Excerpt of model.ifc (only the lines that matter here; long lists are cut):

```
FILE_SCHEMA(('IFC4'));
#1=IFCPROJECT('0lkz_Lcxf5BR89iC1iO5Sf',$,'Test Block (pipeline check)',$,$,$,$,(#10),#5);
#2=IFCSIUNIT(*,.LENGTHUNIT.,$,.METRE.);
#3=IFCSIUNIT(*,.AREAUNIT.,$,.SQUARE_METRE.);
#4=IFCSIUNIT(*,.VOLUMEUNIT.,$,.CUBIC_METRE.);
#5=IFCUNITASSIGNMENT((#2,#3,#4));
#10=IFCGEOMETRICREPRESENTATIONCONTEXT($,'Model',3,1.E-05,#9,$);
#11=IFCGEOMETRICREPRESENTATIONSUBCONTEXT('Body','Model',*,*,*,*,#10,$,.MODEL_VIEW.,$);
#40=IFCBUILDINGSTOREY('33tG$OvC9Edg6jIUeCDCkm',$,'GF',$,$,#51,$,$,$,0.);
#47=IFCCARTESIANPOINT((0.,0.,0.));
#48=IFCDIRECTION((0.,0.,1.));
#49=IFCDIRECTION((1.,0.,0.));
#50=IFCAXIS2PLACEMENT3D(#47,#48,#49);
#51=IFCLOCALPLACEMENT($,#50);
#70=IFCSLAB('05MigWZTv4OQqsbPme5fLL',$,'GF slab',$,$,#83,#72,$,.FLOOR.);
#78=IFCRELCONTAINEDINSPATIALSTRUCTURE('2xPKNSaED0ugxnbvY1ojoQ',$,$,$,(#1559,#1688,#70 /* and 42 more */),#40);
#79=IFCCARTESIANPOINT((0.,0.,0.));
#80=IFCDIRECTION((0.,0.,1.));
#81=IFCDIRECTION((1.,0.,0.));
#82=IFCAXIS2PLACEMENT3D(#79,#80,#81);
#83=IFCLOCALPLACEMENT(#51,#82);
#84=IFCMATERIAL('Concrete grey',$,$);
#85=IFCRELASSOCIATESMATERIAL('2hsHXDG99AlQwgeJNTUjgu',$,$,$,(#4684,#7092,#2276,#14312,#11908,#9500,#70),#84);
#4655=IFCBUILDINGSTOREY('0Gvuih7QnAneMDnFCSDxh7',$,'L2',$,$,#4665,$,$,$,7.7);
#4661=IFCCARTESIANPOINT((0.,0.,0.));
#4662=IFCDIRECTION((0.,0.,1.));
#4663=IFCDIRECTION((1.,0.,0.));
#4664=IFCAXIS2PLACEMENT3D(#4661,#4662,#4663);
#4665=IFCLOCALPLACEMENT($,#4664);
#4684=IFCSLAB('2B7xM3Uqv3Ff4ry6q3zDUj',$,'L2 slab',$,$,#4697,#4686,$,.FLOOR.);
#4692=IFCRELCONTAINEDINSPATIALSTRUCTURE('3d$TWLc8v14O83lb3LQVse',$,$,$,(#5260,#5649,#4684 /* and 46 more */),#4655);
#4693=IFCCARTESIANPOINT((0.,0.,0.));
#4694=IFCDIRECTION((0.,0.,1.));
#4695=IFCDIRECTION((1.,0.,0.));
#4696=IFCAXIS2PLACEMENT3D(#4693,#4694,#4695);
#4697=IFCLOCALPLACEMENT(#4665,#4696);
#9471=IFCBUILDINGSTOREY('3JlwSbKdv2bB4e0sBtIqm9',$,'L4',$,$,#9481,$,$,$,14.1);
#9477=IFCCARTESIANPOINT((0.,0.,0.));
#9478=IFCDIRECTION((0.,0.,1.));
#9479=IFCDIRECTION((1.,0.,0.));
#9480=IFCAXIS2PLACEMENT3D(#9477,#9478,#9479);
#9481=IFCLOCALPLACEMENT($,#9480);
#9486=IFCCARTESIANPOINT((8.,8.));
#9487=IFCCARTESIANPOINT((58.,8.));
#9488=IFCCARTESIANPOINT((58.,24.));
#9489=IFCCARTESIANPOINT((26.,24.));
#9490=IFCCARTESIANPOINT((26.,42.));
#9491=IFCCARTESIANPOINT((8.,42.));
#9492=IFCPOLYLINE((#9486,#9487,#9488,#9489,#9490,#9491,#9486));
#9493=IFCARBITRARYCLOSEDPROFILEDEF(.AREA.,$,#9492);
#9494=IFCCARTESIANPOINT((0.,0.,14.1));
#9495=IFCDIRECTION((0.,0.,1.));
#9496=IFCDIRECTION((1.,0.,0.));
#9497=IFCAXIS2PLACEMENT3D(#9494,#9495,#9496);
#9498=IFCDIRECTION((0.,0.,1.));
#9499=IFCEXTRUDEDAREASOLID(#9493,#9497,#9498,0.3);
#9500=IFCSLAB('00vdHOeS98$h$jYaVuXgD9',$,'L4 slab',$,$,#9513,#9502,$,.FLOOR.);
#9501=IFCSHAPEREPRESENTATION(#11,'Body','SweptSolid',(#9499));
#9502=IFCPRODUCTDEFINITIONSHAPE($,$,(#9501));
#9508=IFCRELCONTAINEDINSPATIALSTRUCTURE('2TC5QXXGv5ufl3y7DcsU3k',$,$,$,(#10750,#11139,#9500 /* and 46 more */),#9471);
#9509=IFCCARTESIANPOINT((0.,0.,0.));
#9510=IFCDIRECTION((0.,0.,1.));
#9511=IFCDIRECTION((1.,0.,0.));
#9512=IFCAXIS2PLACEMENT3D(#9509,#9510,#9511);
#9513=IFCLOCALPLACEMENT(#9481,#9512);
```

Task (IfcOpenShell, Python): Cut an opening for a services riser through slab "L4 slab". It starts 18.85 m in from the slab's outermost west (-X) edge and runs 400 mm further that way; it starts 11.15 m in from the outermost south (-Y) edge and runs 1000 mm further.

```python
import numpy as np
import ifcopenshell
import ifcopenshell.api.feature
import ifcopenshell.api.geometry
import ifcopenshell.api.root
import ifcopenshell.geom
import ifcopenshell.util.placement
import ifcopenshell.util.representation
import ifcopenshell.util.shape
import ifcopenshell.util.unit

model = ifcopenshell.open("model.ifc")
unit_scale = ifcopenshell.util.unit.calculate_unit_scale(model)
settings = ifcopenshell.geom.settings()


def volume(element):
    """Net volume in cubic metres, openings subtracted."""
    shape = ifcopenshell.geom.create_shape(settings, element)
    return ifcopenshell.util.shape.get_volume(shape.geometry)


slab = model.by_id(9500)
before = volume(slab)

# Extent in the slab's own axes, in metres. The edges named are its -X and -Y sides.
slab_shape = ifcopenshell.geom.create_shape(settings, slab)
vertices = ifcopenshell.util.shape.get_vertices(slab_shape.geometry)
x_min, y_min, bottom = vertices.min(axis=0)
top = vertices[:, 2].max()

opening = ifcopenshell.api.root.create_entity(model, ifc_class="IfcOpeningElement", name="Services riser opening", predefined_type="OPENING")
context = ifcopenshell.util.representation.get_context(model, "Model", "Body", "MODEL_VIEW")
width, depth = 0.4, 1
outline = [(0.0, 0.0), (width, 0.0), (width, depth), (0.0, depth), (0.0, 0.0)]
# Overshoot both faces by 50 mm so the cut is clean.
shape = ifcopenshell.api.geometry.add_slab_representation(
    model, context=context, depth=top - bottom + 0.1, polyline=outline
)
ifcopenshell.api.geometry.assign_representation(model, product=opening, representation=shape)

matrix = ifcopenshell.util.placement.get_local_placement(slab.ObjectPlacement)
matrix[:, 3] = matrix @ np.append(np.array([x_min + 18.85, y_min + 11.15, bottom - 0.05]) / unit_scale, 1.0)
ifcopenshell.api.geometry.edit_object_placement(model, product=opening, matrix=matrix, is_si=False)
ifcopenshell.api.feature.add_feature(model, feature=opening, element=slab)

after = volume(slab)

print(f"slab volume {before:.3f} -> {after:.3f} m3")

model.write("model_edited.ifc")
```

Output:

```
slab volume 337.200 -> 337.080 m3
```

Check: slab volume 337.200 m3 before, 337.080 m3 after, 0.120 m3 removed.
